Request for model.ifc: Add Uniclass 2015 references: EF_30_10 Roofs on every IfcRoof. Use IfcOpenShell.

First a look at what the model holds.

```python
import ifcopenshell

model = ifcopenshell.open("model.ifc")
print(model.schema)
print("classifications:", [c.Name for c in model.by_type("IfcClassification")])
for ifc_class in ("IfcDoor", "IfcRoof", "IfcStair", "IfcWall", "IfcWindow"):
    print(ifc_class, len(model.by_type(ifc_class)))
```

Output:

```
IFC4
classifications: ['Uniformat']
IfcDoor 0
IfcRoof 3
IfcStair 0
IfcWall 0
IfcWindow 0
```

```python
import ifcopenshell
import ifcopenshell.api.classification

model = ifcopenshell.open("model.ifc")

system = ifcopenshell.api.classification.add_classification(model, classification="Uniclass 2015")

codes = {
    "IfcRoof": ("EF_30_10", "Roofs"),
}
for ifc_class, (code, name) in codes.items():
    products = model.by_type(ifc_class)
    ifcopenshell.api.classification.add_reference(
        model, products=products, classification=system, identification=code, name=name
    )
    print(code, len(products))

model.write("model-out.ifc")
```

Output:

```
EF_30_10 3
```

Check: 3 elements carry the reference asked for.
